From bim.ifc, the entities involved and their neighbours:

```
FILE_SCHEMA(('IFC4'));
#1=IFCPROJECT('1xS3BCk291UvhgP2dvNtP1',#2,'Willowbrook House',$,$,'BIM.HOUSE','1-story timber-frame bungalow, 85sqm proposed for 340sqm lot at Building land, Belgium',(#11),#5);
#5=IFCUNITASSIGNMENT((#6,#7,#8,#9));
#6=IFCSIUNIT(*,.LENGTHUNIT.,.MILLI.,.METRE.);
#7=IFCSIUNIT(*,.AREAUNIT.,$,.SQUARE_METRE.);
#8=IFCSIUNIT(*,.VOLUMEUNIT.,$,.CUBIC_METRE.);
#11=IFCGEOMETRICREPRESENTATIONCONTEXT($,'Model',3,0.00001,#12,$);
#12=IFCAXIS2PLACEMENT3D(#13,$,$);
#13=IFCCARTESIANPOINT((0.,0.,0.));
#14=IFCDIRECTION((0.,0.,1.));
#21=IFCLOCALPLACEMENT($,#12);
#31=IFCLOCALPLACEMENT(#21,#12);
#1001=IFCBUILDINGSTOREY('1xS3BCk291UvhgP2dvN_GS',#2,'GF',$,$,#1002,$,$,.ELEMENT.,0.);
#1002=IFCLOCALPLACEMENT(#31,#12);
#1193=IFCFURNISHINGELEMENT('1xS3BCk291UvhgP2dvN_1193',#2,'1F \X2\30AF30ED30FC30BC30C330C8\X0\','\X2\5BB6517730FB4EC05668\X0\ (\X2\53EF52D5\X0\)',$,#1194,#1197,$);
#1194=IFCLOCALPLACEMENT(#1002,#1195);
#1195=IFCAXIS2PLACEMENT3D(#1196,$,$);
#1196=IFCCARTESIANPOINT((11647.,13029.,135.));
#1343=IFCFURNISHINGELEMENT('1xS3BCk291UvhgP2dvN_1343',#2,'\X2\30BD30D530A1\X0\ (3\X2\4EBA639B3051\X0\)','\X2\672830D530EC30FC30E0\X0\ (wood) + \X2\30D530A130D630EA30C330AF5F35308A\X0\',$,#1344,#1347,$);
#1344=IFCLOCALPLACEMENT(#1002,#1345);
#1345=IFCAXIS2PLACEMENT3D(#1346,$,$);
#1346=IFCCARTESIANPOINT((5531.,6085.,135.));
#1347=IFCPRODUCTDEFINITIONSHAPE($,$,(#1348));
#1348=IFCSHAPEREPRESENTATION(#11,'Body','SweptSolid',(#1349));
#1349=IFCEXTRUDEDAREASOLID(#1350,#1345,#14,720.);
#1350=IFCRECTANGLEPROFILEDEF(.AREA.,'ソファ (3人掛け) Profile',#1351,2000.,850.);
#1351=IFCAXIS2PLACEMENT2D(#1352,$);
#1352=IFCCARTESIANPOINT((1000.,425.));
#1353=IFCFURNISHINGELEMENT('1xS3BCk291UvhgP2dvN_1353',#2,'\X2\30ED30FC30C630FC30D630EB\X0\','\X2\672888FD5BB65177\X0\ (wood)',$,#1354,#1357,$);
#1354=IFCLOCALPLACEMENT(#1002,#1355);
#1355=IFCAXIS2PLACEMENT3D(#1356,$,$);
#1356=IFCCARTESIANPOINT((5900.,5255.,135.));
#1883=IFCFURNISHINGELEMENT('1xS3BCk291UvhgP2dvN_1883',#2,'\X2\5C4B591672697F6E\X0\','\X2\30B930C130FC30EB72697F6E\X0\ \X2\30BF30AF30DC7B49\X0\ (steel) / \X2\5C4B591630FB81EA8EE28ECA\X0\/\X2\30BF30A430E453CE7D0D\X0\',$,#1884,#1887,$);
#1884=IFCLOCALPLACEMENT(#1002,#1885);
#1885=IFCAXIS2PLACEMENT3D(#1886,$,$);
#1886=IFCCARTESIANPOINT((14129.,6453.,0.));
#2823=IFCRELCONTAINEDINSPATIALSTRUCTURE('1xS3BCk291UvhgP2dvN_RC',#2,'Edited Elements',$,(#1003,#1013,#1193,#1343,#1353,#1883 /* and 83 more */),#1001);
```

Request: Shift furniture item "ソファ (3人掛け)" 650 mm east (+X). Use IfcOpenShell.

```python
import ifcopenshell
import ifcopenshell.api.geometry
import ifcopenshell.util.placement
import ifcopenshell.util.unit

model = ifcopenshell.open("bim.ifc")
unit_scale = ifcopenshell.util.unit.calculate_unit_scale(model)

item = model.by_guid("1xS3BCk291UvhgP2dvN_1343")
matrix = ifcopenshell.util.placement.get_local_placement(item.ObjectPlacement)
matrix[0, 3] += 0.65 / unit_scale
ifcopenshell.api.geometry.edit_object_placement(model, product=item, matrix=matrix, is_si=False)

print(ifcopenshell.util.placement.get_local_placement(item.ObjectPlacement).round(3) + 0.0)

model.write("bim_v2.ifc")
```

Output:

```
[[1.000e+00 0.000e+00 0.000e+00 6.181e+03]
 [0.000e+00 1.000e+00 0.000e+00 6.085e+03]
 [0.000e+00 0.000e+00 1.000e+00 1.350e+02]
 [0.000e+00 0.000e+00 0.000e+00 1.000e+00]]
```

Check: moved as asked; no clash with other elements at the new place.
